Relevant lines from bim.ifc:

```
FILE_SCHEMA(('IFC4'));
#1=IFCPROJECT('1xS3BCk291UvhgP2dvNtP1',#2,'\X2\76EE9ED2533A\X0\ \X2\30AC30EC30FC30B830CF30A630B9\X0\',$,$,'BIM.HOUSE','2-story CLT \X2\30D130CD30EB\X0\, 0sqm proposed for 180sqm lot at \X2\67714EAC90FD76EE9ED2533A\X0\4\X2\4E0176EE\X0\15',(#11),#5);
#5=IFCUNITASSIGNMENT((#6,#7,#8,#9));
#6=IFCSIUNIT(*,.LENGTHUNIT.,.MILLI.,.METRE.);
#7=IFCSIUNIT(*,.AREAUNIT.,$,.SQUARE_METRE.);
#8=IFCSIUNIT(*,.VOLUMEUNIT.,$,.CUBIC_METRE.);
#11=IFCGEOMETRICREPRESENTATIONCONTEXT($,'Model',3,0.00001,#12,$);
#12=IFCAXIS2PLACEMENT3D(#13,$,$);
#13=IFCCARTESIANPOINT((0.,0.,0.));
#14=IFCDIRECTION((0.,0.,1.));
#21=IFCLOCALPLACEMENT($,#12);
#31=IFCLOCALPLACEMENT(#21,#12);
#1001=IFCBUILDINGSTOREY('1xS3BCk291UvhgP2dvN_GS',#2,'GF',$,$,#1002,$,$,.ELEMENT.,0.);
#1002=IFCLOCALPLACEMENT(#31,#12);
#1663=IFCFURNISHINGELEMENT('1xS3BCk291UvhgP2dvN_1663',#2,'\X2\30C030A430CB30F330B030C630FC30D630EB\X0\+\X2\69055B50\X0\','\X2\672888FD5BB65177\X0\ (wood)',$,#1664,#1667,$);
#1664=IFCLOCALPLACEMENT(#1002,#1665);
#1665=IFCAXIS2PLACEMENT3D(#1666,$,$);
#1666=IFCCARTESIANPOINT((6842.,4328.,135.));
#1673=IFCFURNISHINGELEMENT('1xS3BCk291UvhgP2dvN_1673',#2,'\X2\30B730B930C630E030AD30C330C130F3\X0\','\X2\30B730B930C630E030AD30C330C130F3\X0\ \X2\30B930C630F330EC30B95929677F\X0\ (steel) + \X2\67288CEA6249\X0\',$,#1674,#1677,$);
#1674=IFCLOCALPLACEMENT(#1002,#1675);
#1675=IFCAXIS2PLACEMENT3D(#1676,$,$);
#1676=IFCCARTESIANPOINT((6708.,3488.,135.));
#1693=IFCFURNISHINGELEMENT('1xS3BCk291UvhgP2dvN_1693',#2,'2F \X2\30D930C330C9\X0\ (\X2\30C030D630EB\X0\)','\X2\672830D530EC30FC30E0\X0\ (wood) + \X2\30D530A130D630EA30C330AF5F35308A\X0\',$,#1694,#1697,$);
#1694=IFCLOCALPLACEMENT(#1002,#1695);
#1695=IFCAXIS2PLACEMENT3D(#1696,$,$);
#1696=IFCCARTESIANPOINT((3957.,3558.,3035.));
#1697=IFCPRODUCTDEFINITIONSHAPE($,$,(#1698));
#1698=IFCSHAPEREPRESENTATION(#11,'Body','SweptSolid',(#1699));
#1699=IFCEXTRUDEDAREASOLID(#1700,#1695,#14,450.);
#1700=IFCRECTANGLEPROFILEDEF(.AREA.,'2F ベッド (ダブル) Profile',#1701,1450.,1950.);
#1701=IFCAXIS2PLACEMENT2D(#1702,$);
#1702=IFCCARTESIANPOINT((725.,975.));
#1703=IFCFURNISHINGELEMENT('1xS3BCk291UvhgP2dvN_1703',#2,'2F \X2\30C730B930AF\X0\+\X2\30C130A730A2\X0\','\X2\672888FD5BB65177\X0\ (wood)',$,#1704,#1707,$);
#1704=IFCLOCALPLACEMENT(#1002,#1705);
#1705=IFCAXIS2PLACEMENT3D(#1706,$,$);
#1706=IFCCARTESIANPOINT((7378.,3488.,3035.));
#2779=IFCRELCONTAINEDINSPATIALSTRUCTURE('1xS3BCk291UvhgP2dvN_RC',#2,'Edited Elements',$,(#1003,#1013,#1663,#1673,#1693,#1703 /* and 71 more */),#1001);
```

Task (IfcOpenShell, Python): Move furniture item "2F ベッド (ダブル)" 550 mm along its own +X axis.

```python
import ifcopenshell
import ifcopenshell.api.geometry
import ifcopenshell.util.placement
import ifcopenshell.util.unit

model = ifcopenshell.open("bim.ifc")
unit_scale = ifcopenshell.util.unit.calculate_unit_scale(model)

item = model.by_guid("1xS3BCk291UvhgP2dvN_1693")
matrix = ifcopenshell.util.placement.get_local_placement(item.ObjectPlacement)
matrix[:3, 3] += matrix[:3, 0] * 0.55 / unit_scale
ifcopenshell.api.geometry.edit_object_placement(model, product=item, matrix=matrix, is_si=False)

print(ifcopenshell.util.placement.get_local_placement(item.ObjectPlacement).round(3) + 0.0)

model.write("bim_edited.ifc")
```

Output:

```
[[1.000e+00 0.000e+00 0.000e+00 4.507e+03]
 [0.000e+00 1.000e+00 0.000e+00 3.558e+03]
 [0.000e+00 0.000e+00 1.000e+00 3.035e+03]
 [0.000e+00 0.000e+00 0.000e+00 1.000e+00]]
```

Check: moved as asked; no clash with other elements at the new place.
